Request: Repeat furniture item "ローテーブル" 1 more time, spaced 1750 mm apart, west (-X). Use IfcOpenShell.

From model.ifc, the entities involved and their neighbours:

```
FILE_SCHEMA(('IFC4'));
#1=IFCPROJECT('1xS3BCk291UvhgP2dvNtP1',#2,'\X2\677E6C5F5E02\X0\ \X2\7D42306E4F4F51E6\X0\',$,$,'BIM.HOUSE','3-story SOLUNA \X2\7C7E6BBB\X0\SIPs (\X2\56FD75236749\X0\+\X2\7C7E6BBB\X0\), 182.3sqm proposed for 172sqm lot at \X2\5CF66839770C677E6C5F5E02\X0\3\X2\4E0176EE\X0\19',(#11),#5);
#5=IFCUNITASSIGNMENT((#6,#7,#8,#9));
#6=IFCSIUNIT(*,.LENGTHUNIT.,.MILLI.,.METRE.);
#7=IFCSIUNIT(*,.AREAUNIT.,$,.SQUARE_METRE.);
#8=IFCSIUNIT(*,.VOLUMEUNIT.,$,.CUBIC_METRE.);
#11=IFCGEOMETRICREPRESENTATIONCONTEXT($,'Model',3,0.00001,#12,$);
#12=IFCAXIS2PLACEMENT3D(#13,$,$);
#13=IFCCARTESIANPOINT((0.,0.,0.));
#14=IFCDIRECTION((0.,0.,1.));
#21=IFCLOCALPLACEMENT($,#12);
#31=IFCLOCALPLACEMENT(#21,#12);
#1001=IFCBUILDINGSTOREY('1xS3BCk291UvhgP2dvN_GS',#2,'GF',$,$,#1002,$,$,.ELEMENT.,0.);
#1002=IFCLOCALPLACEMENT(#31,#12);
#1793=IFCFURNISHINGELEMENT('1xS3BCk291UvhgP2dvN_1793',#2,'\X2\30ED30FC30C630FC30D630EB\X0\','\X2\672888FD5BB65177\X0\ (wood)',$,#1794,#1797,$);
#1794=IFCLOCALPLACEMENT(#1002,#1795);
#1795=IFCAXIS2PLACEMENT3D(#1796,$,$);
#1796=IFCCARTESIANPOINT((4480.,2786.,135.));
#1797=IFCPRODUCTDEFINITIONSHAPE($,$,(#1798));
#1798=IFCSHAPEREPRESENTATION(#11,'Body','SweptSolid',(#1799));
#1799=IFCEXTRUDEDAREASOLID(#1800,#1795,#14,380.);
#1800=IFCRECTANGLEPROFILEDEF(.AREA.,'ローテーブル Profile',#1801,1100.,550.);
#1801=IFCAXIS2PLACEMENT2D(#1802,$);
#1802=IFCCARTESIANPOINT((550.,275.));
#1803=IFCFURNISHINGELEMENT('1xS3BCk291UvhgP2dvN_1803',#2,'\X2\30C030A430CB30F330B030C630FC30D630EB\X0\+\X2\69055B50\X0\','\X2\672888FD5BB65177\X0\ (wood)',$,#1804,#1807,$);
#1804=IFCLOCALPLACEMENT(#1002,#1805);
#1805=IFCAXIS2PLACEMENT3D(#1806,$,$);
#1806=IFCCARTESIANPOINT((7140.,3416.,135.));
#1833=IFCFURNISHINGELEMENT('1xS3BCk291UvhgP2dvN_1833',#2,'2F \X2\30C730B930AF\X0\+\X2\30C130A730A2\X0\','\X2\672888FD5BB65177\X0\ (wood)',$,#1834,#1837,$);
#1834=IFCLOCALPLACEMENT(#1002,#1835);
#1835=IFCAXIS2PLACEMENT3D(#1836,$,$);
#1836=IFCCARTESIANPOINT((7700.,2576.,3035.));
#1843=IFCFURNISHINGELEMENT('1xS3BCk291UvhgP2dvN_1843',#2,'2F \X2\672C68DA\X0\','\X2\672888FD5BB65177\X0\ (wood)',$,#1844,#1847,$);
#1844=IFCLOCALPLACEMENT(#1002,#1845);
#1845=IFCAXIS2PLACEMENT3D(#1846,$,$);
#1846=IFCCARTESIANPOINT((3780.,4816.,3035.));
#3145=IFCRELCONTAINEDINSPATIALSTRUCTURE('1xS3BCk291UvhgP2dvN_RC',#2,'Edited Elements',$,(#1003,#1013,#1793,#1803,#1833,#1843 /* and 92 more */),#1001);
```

```python
import numpy as np
import ifcopenshell
import ifcopenshell.api.geometry
import ifcopenshell.api.root
import ifcopenshell.util.element
import ifcopenshell.util.placement
import ifcopenshell.util.unit

model = ifcopenshell.open("model.ifc")
unit_scale = ifcopenshell.util.unit.calculate_unit_scale(model)


def reuse_history(source, copy):
    """copy_class also copies each property set's owner history, people and application; keep the originals."""
    for rel in copy.IsDefinedBy:
        if rel.is_a("IfcRelDefinesByProperties") and (history := rel.RelatingPropertyDefinition.OwnerHistory):
            rel.RelatingPropertyDefinition.OwnerHistory = source.OwnerHistory
            ifcopenshell.util.element.remove_deep2(model, history)


source = model.by_guid("1xS3BCk291UvhgP2dvN_1793")
base = ifcopenshell.util.placement.get_local_placement(source.ObjectPlacement)
step = np.array([-1.0, 0.0, 0.0]) * 1.75 / unit_scale

for i in range(1, 2):
    copy = ifcopenshell.api.root.copy_class(model, product=source)
    copy.Representation = ifcopenshell.util.element.copy_deep(
        model, source.Representation, exclude=["IfcGeometricRepresentationContext", "IfcRepresentationMap"]
    )
    reuse_history(source, copy)
    matrix = base.copy()
    matrix[:3, 3] += i * step
    print("added at", matrix[:3, 3].round(3) + 0.0)
    ifcopenshell.api.geometry.edit_object_placement(model, product=copy, matrix=matrix, is_si=False)

model.write("model_edited.ifc")
```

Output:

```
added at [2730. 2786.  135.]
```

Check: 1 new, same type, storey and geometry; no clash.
